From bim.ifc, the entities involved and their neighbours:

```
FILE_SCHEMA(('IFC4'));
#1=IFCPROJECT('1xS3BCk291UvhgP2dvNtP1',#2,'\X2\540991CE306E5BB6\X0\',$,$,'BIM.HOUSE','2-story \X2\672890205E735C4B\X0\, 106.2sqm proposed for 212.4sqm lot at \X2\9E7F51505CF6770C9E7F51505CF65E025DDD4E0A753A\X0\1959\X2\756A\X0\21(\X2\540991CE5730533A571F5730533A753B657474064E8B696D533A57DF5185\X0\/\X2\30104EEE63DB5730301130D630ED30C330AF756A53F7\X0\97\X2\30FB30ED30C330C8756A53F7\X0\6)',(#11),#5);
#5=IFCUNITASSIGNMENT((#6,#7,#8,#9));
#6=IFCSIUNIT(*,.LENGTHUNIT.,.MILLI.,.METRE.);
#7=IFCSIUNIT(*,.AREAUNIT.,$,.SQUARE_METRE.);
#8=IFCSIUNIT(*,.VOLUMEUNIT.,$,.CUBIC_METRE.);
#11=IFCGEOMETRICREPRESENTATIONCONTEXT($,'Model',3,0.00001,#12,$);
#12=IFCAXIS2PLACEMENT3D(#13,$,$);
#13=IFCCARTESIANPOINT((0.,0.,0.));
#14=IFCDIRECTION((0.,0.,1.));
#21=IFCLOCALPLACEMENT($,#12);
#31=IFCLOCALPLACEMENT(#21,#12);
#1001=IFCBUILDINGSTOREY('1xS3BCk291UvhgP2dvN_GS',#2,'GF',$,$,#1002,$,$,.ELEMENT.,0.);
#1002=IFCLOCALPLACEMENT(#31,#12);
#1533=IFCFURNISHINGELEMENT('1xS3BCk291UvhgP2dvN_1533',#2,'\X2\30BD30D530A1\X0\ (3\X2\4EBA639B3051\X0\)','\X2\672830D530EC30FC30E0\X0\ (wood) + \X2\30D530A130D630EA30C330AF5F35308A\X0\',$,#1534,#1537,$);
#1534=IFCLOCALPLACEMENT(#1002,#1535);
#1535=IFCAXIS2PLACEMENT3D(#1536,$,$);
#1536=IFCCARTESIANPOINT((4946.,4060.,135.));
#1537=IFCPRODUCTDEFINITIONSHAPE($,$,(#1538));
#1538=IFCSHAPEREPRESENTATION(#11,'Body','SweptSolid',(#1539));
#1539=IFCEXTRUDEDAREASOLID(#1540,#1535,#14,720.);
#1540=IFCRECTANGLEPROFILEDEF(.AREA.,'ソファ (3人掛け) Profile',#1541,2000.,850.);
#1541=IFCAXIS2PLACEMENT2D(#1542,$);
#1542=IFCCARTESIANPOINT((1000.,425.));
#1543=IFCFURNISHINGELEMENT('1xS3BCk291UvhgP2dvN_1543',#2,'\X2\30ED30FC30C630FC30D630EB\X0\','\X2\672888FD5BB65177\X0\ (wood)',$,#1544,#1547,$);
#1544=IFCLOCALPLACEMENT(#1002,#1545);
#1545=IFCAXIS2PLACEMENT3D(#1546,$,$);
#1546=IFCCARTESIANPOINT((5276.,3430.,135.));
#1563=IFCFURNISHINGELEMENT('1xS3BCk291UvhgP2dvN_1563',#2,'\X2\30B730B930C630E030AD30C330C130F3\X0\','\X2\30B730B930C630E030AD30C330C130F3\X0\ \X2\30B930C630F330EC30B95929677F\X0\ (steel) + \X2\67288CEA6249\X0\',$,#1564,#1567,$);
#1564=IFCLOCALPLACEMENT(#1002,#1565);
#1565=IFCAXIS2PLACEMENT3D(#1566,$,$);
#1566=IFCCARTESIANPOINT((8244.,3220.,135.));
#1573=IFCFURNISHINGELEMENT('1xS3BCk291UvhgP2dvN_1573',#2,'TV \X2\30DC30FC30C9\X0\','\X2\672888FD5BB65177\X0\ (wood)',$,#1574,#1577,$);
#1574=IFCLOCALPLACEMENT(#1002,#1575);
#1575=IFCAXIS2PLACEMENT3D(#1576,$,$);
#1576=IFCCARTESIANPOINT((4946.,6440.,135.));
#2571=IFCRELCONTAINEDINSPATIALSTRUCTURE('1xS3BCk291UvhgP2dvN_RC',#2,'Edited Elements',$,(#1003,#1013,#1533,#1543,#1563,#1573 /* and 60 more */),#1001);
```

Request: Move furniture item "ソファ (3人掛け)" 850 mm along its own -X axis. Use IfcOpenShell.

```python
import ifcopenshell
import ifcopenshell.api.geometry
import ifcopenshell.util.placement
import ifcopenshell.util.unit

model = ifcopenshell.open("bim.ifc")
unit_scale = ifcopenshell.util.unit.calculate_unit_scale(model)

item = model.by_id(1533)
matrix = ifcopenshell.util.placement.get_local_placement(item.ObjectPlacement)
matrix[:3, 3] -= matrix[:3, 0] * 0.85 / unit_scale
ifcopenshell.api.geometry.edit_object_placement(model, product=item, matrix=matrix, is_si=False)

print(ifcopenshell.util.placement.get_local_placement(item.ObjectPlacement).round(3) + 0.0)

model.write("bim-out.ifc")
```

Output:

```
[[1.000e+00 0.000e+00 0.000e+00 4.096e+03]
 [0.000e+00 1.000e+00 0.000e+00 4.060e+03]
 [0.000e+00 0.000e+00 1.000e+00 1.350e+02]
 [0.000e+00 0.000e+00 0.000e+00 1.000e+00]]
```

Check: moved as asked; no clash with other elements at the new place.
